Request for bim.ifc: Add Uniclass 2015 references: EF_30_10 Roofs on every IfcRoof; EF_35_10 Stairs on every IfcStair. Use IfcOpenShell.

First a look at what the model holds.

```python
import ifcopenshell

model = ifcopenshell.open("bim.ifc")
print(model.schema)
print("classifications:", [c.Name for c in model.by_type("IfcClassification")])
for ifc_class in ("IfcDoor", "IfcRoof", "IfcStair", "IfcWall", "IfcWindow"):
    print(ifc_class, len(model.by_type(ifc_class)))
```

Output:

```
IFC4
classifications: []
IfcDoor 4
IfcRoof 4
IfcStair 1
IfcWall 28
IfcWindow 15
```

```python
import ifcopenshell
import ifcopenshell.api.classification

model = ifcopenshell.open("bim.ifc")

system = ifcopenshell.api.classification.add_classification(model, classification="Uniclass 2015")

codes = {
    "IfcRoof": ("EF_30_10", "Roofs"),
    "IfcStair": ("EF_35_10", "Stairs"),
}
for ifc_class, (code, name) in codes.items():
    products = model.by_type(ifc_class)
    ifcopenshell.api.classification.add_reference(
        model, products=products, classification=system, identification=code, name=name
    )
    print(code, len(products))

model.write("bim-out.ifc")
```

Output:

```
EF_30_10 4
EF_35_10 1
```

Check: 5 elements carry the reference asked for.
